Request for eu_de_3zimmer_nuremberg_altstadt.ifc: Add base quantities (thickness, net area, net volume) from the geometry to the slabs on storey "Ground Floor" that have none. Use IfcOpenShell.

First a look at what the model holds.

```python
import ifcopenshell
import ifcopenshell.util.element
import ifcopenshell.util.unit

model = ifcopenshell.open("eu_de_3zimmer_nuremberg_altstadt.ifc")
print(model.schema)
for unit_type in ("LENGTHUNIT", "AREAUNIT", "VOLUMEUNIT"):
    print(unit_type, ifcopenshell.util.unit.calculate_unit_scale(model, unit_type))
storey = next(s for s in model.by_type("IfcBuildingStorey") if s.Name == "Ground Floor")
slabs = [e for e in ifcopenshell.util.element.get_decomposition(storey) if e.is_a("IfcSlab")]
for e in sorted(slabs, key=lambda e: e.id()):
    print(e.id(), e.is_a(), e.Name, list(ifcopenshell.util.element.get_psets(e, qtos_only=True)), sep=" | ")
```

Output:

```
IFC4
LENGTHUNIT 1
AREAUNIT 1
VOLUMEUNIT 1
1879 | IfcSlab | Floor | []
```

```python
import ifcopenshell
import ifcopenshell.api.pset
import ifcopenshell.geom
import ifcopenshell.util.element
import ifcopenshell.util.shape
import ifcopenshell.util.unit

model = ifcopenshell.open("eu_de_3zimmer_nuremberg_altstadt.ifc")
unit_scale = ifcopenshell.util.unit.calculate_unit_scale(model)
area_scale = ifcopenshell.util.unit.calculate_unit_scale(model, "AREAUNIT")
volume_scale = ifcopenshell.util.unit.calculate_unit_scale(model, "VOLUMEUNIT")
settings = ifcopenshell.geom.settings()

storey = next(s for s in model.by_type("IfcBuildingStorey") if s.Name == "Ground Floor")
slabs = [e for e in ifcopenshell.util.element.get_decomposition(storey) if e.is_a("IfcSlab")]

for e in sorted(slabs, key=lambda e: e.id()):
    if ifcopenshell.util.element.get_psets(e, qtos_only=True, should_inherit=False):
        continue
    # Geometry comes back in metres, in the element's own axes.
    shape = ifcopenshell.geom.create_shape(settings, e)
    values = {
        "Width": ifcopenshell.util.shape.get_z(shape.geometry) / unit_scale,
        "NetArea": ifcopenshell.util.shape.get_footprint_area(shape.geometry) / area_scale,
        "NetVolume": ifcopenshell.util.shape.get_volume(shape.geometry) / volume_scale,
    }
    qto = ifcopenshell.api.pset.add_qto(model, product=e, name="Qto_SlabBaseQuantities")
    ifcopenshell.api.pset.edit_qto(model, qto=qto, properties=values)
    print(e.id(), {k: round(v, 3) for k, v in values.items()})

model.write("eu_de_3zimmer_nuremberg_altstadt_rev.ifc")
```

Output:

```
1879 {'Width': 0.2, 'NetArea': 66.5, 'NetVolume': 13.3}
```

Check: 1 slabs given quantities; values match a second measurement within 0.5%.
